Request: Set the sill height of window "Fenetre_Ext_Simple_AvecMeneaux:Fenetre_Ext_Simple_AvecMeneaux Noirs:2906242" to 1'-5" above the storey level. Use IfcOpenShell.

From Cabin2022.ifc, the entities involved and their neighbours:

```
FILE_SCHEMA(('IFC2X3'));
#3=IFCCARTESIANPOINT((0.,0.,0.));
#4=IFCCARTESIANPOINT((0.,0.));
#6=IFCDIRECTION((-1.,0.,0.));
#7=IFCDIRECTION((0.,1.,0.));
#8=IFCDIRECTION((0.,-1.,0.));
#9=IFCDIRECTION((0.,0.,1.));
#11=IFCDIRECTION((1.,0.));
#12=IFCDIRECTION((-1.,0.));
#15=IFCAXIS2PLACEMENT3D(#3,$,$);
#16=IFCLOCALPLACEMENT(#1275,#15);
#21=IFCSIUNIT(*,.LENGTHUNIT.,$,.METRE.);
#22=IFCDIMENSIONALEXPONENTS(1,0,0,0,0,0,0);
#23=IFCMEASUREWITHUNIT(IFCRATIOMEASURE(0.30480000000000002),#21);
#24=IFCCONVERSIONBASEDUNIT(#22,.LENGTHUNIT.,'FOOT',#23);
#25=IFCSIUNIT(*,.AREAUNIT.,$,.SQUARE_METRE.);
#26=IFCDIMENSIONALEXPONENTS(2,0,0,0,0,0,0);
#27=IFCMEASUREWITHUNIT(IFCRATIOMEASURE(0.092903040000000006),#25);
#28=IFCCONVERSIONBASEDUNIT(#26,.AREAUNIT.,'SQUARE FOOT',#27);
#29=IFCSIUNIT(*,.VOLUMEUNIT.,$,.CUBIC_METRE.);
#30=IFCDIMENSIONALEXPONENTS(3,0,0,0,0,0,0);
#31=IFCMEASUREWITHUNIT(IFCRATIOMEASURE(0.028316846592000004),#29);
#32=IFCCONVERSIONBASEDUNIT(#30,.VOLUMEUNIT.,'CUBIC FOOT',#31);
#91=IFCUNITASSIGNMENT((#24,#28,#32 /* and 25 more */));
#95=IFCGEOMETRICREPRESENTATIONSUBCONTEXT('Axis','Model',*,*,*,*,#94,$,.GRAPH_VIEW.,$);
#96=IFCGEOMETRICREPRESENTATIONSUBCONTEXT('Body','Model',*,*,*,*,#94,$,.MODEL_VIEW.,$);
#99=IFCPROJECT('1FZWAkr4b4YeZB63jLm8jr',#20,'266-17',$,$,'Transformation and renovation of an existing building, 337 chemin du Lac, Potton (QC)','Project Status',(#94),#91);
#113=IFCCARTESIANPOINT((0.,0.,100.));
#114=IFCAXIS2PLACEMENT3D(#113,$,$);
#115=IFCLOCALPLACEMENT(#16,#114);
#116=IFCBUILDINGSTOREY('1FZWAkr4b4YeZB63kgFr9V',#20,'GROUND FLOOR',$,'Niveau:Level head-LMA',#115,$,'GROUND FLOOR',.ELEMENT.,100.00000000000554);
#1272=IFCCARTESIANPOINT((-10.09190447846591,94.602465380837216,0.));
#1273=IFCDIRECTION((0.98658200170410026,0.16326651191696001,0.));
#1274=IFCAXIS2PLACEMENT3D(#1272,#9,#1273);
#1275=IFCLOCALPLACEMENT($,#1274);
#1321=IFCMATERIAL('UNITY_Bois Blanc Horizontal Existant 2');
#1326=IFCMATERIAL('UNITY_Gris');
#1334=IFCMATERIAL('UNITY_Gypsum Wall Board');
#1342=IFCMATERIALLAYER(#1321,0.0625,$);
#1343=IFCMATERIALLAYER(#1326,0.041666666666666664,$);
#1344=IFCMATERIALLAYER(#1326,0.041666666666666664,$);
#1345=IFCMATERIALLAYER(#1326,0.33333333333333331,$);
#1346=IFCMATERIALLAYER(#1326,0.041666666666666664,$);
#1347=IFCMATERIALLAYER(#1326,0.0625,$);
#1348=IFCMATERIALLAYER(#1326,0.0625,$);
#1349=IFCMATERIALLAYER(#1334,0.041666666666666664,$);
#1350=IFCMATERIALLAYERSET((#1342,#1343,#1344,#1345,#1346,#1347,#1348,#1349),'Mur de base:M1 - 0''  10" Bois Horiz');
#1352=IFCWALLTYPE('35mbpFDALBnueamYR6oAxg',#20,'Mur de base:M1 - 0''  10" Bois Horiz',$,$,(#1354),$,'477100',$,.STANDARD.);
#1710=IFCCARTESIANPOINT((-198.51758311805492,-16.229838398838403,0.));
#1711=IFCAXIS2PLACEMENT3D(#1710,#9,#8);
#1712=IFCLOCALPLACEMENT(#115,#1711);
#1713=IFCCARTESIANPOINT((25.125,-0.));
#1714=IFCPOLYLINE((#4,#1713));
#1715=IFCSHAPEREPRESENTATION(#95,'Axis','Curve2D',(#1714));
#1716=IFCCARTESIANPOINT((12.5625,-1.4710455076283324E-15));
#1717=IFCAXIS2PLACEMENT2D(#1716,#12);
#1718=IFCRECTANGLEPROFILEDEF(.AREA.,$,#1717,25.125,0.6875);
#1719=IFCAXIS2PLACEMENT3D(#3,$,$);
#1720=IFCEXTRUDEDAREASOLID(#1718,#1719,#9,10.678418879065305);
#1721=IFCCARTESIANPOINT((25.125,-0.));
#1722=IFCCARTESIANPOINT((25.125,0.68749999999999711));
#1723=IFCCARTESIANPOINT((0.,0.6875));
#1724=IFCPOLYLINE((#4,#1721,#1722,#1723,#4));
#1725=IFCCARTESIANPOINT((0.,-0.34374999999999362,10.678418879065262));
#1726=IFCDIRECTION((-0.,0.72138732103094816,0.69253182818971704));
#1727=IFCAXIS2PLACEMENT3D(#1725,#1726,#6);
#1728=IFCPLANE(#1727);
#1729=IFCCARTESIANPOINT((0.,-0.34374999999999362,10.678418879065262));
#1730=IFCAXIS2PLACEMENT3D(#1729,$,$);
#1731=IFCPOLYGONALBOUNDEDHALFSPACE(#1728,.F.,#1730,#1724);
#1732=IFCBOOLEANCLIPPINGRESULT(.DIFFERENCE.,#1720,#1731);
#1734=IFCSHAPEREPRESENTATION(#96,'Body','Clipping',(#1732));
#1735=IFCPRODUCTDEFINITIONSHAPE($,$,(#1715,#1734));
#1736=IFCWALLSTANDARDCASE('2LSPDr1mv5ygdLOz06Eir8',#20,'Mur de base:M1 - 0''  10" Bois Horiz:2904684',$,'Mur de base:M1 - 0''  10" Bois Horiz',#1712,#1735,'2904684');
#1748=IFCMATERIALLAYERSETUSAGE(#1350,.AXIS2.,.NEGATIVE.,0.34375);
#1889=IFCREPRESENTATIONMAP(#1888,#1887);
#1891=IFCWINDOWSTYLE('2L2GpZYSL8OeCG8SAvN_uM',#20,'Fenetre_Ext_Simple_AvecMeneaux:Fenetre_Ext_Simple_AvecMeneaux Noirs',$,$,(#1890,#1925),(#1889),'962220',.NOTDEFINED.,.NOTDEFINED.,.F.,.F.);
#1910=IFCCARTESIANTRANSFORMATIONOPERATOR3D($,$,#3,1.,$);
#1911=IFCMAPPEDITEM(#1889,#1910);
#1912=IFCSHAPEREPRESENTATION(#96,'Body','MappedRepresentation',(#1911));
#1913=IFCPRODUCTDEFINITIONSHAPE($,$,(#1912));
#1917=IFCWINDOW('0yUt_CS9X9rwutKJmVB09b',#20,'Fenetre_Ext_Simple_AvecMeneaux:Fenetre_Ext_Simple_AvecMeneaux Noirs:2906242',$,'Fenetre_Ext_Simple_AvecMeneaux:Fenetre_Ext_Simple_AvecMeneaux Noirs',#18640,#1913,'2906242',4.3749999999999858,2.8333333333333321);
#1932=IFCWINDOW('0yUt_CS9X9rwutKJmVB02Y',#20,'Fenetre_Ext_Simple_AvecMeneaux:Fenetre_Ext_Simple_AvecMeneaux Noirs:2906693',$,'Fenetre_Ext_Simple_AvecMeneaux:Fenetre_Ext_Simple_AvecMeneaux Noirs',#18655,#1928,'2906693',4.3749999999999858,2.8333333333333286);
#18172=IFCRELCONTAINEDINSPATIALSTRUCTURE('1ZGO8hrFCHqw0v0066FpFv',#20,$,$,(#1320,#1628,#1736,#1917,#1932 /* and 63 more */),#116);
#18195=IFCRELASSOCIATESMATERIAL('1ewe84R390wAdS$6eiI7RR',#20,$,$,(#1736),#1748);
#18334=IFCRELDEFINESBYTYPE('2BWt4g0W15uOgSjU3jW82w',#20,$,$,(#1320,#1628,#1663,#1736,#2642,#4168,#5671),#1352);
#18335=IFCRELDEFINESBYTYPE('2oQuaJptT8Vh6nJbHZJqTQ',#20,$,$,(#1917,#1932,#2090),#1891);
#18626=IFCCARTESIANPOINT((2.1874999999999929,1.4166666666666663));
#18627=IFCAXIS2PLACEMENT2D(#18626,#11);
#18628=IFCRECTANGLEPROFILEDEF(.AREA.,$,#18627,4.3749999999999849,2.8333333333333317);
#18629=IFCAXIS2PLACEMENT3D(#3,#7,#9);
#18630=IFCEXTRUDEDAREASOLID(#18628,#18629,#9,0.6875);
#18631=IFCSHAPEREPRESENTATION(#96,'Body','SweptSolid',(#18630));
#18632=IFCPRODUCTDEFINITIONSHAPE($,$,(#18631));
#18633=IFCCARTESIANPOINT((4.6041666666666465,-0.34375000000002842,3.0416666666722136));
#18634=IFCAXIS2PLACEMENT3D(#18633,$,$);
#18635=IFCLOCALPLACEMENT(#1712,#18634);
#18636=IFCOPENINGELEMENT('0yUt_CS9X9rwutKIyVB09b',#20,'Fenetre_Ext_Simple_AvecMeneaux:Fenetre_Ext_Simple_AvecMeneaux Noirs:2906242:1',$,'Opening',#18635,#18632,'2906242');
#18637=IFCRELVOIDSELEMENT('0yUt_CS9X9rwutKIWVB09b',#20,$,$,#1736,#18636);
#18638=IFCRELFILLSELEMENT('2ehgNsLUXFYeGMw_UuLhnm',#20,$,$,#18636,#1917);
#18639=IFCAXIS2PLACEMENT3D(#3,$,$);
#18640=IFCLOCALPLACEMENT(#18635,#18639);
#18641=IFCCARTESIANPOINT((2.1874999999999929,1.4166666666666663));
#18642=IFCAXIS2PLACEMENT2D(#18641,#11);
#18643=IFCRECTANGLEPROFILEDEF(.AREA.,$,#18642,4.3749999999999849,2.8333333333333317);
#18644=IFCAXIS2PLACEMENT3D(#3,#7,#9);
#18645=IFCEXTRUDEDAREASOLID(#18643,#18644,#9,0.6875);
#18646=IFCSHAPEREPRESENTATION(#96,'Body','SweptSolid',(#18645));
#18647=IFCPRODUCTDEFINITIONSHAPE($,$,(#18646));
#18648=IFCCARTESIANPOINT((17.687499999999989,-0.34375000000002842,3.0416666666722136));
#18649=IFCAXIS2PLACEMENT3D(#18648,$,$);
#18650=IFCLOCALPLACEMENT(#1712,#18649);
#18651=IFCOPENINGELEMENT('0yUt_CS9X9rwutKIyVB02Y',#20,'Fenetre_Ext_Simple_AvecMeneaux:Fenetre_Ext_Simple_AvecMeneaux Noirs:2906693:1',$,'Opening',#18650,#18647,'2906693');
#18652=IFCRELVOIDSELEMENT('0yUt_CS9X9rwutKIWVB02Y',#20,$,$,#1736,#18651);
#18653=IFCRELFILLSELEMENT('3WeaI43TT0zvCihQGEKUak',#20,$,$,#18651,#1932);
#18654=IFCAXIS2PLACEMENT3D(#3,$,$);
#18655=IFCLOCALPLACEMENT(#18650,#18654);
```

```python
import numpy as np
import ifcopenshell
import ifcopenshell.api.geometry
import ifcopenshell.geom
import ifcopenshell.util.element
import ifcopenshell.util.placement
import ifcopenshell.util.shape
import ifcopenshell.util.unit

model = ifcopenshell.open("Cabin2022.ifc")
unit_scale = ifcopenshell.util.unit.calculate_unit_scale(model)

window = model.by_id(1917)
opening = window.FillsVoids[0].RelatingOpeningElement
storey = ifcopenshell.util.element.get_container(window, ifc_class="IfcBuildingStorey")
level = ifcopenshell.util.placement.get_local_placement(storey.ObjectPlacement)[2, 3]

# The opening's origin need not be at the sill, so measure its lowest point.
shape = ifcopenshell.geom.create_shape(ifcopenshell.geom.settings(), opening)
bottom = ifcopenshell.util.shape.get_shape_bottom_elevation(shape, shape.geometry) / unit_scale
dz = level + 17 * 0.0254 / unit_scale - bottom

shift = np.array([0.0, 0.0, dz])
# The window is placed relative to its opening, so it follows when the opening moves.
matrix = ifcopenshell.util.placement.get_local_placement(opening.ObjectPlacement)
matrix[:3, 3] += shift
ifcopenshell.api.geometry.edit_object_placement(
    model, product=opening, matrix=matrix, is_si=False, should_transform_children=True
)

print(f"moved by {dz * unit_scale:+.3f} m")

model.write("Cabin2022_rev.ifc")
```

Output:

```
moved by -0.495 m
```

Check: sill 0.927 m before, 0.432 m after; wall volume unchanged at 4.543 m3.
